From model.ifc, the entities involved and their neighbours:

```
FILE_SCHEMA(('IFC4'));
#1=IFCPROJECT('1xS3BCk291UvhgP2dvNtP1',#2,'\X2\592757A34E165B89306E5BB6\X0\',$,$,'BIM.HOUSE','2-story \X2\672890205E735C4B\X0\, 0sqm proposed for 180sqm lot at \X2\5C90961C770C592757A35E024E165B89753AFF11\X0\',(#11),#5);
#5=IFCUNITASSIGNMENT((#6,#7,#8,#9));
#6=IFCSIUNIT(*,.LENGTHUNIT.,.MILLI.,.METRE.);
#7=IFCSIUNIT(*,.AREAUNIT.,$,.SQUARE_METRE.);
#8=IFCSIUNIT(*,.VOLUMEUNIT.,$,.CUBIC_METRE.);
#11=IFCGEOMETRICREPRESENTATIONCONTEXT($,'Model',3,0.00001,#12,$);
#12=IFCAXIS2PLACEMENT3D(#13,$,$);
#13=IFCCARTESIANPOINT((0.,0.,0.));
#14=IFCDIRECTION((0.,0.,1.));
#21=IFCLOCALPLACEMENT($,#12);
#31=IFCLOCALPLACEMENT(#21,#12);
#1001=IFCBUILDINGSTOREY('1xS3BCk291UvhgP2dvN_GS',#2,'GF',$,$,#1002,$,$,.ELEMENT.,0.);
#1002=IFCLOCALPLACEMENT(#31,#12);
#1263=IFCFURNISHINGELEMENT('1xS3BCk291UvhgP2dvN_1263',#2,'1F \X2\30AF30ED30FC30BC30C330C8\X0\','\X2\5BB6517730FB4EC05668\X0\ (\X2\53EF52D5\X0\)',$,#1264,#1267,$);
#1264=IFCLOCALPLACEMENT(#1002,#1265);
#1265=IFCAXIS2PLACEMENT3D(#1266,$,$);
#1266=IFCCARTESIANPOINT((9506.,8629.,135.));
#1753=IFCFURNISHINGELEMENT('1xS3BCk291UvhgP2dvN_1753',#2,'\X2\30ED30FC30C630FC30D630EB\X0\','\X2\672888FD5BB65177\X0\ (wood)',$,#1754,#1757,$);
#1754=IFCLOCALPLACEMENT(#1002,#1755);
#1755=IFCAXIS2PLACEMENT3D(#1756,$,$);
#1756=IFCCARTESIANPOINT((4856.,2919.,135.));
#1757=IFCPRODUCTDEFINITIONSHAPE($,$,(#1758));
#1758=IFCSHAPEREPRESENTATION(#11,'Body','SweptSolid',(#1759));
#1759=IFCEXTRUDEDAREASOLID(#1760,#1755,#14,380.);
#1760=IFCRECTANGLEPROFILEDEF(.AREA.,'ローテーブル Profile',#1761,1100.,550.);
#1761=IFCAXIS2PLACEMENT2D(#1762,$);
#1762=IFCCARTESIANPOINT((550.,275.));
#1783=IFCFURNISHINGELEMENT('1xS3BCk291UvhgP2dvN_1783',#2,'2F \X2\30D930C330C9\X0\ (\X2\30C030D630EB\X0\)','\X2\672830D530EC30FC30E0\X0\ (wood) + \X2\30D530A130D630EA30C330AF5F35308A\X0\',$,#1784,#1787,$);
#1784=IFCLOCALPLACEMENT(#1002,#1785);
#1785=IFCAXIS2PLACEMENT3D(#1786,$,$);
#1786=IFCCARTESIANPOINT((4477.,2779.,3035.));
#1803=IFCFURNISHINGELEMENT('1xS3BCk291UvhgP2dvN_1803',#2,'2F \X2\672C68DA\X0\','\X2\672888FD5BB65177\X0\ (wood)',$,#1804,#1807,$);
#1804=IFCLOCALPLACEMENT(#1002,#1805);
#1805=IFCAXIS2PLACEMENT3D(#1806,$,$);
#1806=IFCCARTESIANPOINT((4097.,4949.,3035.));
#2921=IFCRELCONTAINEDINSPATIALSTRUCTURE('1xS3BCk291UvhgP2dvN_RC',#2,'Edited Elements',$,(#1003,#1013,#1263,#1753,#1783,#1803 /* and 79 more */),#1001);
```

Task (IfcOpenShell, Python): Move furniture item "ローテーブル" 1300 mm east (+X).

```python
import ifcopenshell
import ifcopenshell.api.geometry
import ifcopenshell.util.placement

model = ifcopenshell.open("model.ifc")

item = model.by_guid("1xS3BCk291UvhgP2dvN_1753")
matrix = ifcopenshell.util.placement.get_local_placement(item.ObjectPlacement)
matrix[0, 3] += 1300.0
ifcopenshell.api.geometry.edit_object_placement(model, product=item, matrix=matrix, is_si=False)

print(ifcopenshell.util.placement.get_local_placement(item.ObjectPlacement).round(3) + 0.0)

model.write("model_v2.ifc")
```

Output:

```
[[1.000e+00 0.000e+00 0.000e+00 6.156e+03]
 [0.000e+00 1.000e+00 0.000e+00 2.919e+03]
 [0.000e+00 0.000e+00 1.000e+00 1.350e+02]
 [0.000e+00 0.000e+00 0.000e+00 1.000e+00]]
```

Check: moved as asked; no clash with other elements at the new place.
